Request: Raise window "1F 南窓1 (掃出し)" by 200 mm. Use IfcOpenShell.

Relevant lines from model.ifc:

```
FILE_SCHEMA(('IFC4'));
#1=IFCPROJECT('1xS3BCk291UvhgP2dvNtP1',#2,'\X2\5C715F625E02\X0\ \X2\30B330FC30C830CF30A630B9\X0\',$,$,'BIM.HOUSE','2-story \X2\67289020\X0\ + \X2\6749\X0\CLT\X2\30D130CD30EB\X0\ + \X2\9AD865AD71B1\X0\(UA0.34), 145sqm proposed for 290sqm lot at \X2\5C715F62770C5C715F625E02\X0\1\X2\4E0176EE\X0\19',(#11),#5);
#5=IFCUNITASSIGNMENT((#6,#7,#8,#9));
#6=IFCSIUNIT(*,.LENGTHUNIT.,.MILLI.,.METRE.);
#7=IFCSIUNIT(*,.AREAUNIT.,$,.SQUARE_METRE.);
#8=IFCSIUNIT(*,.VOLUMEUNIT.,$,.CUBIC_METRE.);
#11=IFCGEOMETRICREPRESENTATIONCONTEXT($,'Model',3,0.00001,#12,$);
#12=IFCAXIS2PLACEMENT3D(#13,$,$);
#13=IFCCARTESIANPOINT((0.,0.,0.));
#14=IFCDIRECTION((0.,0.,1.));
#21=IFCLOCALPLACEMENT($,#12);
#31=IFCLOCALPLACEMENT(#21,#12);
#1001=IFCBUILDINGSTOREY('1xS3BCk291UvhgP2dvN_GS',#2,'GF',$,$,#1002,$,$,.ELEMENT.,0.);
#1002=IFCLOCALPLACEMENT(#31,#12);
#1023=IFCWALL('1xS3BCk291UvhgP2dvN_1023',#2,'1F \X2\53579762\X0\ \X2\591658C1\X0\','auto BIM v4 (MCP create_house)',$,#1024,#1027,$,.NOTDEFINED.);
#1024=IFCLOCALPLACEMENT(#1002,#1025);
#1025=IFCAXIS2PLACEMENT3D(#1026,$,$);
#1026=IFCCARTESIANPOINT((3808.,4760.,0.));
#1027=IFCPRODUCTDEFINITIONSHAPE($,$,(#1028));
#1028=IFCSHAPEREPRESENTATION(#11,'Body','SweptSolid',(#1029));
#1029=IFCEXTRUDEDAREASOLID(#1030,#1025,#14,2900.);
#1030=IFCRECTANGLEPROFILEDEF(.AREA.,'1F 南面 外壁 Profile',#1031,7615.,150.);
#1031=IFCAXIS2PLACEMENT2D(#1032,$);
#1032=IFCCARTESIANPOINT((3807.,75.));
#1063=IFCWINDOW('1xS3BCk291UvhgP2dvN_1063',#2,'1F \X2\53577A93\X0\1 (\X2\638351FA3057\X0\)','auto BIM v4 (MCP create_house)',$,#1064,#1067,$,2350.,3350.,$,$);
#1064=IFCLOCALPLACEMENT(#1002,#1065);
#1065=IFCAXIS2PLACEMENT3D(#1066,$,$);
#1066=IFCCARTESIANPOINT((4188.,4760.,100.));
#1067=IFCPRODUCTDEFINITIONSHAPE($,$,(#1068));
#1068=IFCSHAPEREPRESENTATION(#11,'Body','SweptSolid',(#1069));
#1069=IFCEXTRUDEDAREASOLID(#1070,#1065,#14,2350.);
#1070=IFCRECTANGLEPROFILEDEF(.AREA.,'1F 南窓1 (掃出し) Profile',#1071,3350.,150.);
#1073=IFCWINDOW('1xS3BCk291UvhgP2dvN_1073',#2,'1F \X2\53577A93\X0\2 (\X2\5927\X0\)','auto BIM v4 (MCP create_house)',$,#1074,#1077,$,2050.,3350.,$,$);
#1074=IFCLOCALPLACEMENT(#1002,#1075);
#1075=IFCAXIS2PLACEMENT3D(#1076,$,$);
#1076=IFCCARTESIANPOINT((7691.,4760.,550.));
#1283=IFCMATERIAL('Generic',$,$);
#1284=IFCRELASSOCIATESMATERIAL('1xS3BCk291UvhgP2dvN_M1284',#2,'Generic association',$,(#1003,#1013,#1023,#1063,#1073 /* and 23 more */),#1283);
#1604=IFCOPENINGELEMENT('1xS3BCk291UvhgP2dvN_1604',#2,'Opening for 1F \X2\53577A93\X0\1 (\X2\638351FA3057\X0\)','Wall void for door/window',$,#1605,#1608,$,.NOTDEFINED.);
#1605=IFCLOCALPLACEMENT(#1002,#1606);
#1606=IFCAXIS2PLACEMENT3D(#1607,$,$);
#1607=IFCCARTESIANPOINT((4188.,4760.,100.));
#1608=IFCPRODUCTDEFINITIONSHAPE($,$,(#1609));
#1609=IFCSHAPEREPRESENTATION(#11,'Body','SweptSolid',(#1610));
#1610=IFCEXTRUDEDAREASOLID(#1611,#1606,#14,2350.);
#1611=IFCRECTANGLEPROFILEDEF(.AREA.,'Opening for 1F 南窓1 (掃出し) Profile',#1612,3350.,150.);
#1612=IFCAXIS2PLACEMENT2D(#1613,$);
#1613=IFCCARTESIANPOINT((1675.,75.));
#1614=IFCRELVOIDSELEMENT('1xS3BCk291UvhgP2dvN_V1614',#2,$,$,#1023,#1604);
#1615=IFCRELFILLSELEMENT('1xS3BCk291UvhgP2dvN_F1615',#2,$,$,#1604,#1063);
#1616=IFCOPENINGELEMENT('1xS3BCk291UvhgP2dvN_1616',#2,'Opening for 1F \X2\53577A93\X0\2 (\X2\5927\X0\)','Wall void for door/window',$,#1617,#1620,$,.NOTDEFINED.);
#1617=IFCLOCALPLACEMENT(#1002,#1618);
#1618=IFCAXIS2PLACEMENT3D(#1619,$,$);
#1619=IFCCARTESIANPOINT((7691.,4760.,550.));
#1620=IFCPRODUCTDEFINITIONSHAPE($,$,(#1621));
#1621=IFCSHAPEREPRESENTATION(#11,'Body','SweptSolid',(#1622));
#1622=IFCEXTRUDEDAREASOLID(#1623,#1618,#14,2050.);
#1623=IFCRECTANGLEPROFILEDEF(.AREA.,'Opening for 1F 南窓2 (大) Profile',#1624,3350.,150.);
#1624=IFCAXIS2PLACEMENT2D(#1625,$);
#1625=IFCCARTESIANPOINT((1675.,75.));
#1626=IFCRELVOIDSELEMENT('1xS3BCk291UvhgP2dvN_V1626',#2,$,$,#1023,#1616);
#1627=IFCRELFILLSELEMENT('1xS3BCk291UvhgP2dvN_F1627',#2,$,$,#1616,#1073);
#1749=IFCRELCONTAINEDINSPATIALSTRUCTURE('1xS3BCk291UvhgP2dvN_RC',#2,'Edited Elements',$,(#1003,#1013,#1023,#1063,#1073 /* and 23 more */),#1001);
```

```python
import numpy as np
import ifcopenshell
import ifcopenshell.api.geometry
import ifcopenshell.util.placement
import ifcopenshell.util.unit

model = ifcopenshell.open("model.ifc")
unit_scale = ifcopenshell.util.unit.calculate_unit_scale(model)

window = model.by_guid("1xS3BCk291UvhgP2dvN_1063")
opening = window.FillsVoids[0].RelatingOpeningElement
dz = 200.0

shift = np.array([0.0, 0.0, dz])
# The window is not placed relative to its opening, so move both.
for product in (opening, window):
    matrix = ifcopenshell.util.placement.get_local_placement(product.ObjectPlacement)
    matrix[:3, 3] += shift
    ifcopenshell.api.geometry.edit_object_placement(model, product=product, matrix=matrix, is_si=False)

print(f"moved by {dz * unit_scale:+.3f} m")

model.write("model_edited.ifc")
```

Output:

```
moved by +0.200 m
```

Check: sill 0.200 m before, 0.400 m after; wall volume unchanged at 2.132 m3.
